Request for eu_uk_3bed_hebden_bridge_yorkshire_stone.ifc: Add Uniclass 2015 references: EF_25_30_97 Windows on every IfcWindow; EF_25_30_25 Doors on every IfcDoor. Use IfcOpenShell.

First a look at what the model holds.

```python
import ifcopenshell

model = ifcopenshell.open("eu_uk_3bed_hebden_bridge_yorkshire_stone.ifc")
print(model.schema)
print("classifications:", [c.Name for c in model.by_type("IfcClassification")])
for ifc_class in ("IfcDoor", "IfcRoof", "IfcStair", "IfcWall", "IfcWindow"):
    print(ifc_class, len(model.by_type(ifc_class)))
```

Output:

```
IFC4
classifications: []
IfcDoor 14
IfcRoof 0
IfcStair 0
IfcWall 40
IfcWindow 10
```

```python
import ifcopenshell
import ifcopenshell.api.classification

model = ifcopenshell.open("eu_uk_3bed_hebden_bridge_yorkshire_stone.ifc")

system = ifcopenshell.api.classification.add_classification(model, classification="Uniclass 2015")

codes = {
    "IfcWindow": ("EF_25_30_97", "Windows"),
    "IfcDoor": ("EF_25_30_25", "Doors"),
}
for ifc_class, (code, name) in codes.items():
    products = model.by_type(ifc_class)
    ifcopenshell.api.classification.add_reference(
        model, products=products, classification=system, identification=code, name=name
    )
    print(code, len(products))

model.write("eu_uk_3bed_hebden_bridge_yorkshire_stone-out.ifc")
```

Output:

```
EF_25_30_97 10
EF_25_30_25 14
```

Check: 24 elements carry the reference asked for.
